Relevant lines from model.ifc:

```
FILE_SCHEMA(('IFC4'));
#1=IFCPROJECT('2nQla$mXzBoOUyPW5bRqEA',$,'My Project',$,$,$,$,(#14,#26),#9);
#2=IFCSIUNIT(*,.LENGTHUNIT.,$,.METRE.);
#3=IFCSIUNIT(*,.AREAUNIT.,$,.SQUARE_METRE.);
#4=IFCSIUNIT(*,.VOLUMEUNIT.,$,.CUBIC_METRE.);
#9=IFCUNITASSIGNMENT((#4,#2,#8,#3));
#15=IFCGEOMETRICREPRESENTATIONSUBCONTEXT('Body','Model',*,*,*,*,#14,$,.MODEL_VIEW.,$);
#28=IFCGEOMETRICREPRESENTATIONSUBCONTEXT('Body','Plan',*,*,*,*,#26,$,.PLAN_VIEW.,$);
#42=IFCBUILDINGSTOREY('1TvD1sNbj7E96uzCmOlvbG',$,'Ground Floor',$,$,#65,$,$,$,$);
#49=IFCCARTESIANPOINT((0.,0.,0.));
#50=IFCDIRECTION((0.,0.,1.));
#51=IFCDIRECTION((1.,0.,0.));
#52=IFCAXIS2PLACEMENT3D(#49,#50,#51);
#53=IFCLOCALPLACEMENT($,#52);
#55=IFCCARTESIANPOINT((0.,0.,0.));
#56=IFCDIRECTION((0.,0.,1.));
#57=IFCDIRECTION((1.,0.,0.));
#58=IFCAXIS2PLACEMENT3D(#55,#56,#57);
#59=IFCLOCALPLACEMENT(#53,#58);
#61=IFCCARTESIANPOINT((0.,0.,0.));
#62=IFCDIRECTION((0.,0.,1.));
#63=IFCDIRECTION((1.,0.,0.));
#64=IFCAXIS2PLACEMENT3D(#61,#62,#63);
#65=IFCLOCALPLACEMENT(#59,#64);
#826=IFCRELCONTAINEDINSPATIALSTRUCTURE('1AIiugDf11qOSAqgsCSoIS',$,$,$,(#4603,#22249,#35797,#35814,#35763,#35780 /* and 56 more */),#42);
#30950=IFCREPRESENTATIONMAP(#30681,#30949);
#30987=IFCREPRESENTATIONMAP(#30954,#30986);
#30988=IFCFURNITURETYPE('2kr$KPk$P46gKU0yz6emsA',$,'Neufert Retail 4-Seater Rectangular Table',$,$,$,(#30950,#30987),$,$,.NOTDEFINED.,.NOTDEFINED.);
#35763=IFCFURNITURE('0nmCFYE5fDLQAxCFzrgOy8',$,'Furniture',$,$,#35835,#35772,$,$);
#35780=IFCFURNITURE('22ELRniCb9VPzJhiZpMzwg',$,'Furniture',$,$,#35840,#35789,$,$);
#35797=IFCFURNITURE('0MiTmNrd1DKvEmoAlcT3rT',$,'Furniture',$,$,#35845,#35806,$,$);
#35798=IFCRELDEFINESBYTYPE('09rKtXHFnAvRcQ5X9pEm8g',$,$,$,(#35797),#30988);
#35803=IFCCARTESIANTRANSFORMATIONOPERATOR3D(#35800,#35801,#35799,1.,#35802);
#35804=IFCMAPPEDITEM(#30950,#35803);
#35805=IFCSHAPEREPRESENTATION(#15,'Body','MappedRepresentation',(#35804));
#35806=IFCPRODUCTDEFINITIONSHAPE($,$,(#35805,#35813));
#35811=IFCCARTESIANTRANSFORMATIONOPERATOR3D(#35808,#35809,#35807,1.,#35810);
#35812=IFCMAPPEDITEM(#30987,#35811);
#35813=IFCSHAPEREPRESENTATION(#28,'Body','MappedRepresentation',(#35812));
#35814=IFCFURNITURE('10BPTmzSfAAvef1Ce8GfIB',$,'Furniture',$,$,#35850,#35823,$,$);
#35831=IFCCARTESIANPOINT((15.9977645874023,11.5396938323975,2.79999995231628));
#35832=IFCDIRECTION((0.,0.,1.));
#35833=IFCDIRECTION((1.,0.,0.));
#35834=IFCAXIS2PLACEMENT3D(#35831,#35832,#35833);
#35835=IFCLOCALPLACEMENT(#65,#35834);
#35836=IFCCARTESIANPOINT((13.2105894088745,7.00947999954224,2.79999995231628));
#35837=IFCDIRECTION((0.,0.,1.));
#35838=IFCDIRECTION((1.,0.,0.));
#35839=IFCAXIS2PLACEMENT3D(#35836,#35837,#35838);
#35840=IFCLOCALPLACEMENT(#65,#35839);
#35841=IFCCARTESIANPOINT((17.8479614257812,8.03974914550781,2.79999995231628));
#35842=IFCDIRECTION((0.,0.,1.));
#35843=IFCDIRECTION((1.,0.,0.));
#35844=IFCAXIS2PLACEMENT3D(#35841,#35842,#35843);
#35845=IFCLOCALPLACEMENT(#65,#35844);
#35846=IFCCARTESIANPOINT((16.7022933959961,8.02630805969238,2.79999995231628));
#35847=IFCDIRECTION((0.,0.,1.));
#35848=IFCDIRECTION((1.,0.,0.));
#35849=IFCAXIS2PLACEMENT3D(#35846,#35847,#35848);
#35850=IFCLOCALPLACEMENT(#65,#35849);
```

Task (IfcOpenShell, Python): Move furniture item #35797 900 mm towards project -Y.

```python
import ifcopenshell
import ifcopenshell.api.geometry
import ifcopenshell.util.placement
import ifcopenshell.util.unit

model = ifcopenshell.open("model.ifc")
unit_scale = ifcopenshell.util.unit.calculate_unit_scale(model)

item = model.by_guid("0MiTmNrd1DKvEmoAlcT3rT")
matrix = ifcopenshell.util.placement.get_local_placement(item.ObjectPlacement)
matrix[1, 3] -= 0.9 / unit_scale
ifcopenshell.api.geometry.edit_object_placement(model, product=item, matrix=matrix, is_si=False)

print(ifcopenshell.util.placement.get_local_placement(item.ObjectPlacement).round(3) + 0.0)

model.write("model_edited.ifc")
```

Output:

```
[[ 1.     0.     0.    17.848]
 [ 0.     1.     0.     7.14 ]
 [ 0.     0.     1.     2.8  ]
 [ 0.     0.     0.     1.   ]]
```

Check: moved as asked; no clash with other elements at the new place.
